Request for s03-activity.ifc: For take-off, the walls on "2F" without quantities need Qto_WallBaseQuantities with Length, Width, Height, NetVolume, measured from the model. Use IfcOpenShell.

First a look at what the model holds.

```python
import ifcopenshell
import ifcopenshell.util.element
import ifcopenshell.util.unit

model = ifcopenshell.open("s03-activity.ifc")
print(model.schema)
for unit_type in ("LENGTHUNIT", "AREAUNIT", "VOLUMEUNIT"):
    print(unit_type, ifcopenshell.util.unit.calculate_unit_scale(model, unit_type))
storey = next(s for s in model.by_type("IfcBuildingStorey") if s.Name == "2F")
walls = [e for e in ifcopenshell.util.element.get_decomposition(storey) if e.is_a("IfcWall")]
for e in sorted(walls, key=lambda e: e.id()):
    print(e.id(), e.is_a(), e.Name, list(ifcopenshell.util.element.get_psets(e, qtos_only=True)), sep=" | ")
```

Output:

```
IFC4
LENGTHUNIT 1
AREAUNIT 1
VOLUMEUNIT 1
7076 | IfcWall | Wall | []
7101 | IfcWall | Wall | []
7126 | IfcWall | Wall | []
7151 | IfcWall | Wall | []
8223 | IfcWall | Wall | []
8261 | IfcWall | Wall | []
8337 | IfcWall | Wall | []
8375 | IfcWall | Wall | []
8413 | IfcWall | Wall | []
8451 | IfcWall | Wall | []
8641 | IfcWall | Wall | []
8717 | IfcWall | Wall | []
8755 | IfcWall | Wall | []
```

```python
import ifcopenshell
import ifcopenshell.api.pset
import ifcopenshell.geom
import ifcopenshell.util.element
import ifcopenshell.util.shape
import ifcopenshell.util.unit

model = ifcopenshell.open("s03-activity.ifc")
unit_scale = ifcopenshell.util.unit.calculate_unit_scale(model)
volume_scale = ifcopenshell.util.unit.calculate_unit_scale(model, "VOLUMEUNIT")
settings = ifcopenshell.geom.settings()

storey = next(s for s in model.by_type("IfcBuildingStorey") if s.Name == "2F")
walls = [e for e in ifcopenshell.util.element.get_decomposition(storey) if e.is_a("IfcWall")]

for e in sorted(walls, key=lambda e: e.id()):
    if ifcopenshell.util.element.get_psets(e, qtos_only=True, should_inherit=False):
        continue
    # Geometry comes back in metres, in the element's own axes.
    shape = ifcopenshell.geom.create_shape(settings, e)
    values = {
        "Length": ifcopenshell.util.shape.get_x(shape.geometry) / unit_scale,
        "Width": ifcopenshell.util.shape.get_y(shape.geometry) / unit_scale,
        "Height": ifcopenshell.util.shape.get_z(shape.geometry) / unit_scale,
        "NetVolume": ifcopenshell.util.shape.get_volume(shape.geometry) / volume_scale,
    }
    qto = ifcopenshell.api.pset.add_qto(model, product=e, name="Qto_WallBaseQuantities")
    ifcopenshell.api.pset.edit_qto(model, qto=qto, properties=values)
    print(e.id(), {k: round(v, 3) for k, v in values.items()})

model.write("s03-activity_edited.ifc")
```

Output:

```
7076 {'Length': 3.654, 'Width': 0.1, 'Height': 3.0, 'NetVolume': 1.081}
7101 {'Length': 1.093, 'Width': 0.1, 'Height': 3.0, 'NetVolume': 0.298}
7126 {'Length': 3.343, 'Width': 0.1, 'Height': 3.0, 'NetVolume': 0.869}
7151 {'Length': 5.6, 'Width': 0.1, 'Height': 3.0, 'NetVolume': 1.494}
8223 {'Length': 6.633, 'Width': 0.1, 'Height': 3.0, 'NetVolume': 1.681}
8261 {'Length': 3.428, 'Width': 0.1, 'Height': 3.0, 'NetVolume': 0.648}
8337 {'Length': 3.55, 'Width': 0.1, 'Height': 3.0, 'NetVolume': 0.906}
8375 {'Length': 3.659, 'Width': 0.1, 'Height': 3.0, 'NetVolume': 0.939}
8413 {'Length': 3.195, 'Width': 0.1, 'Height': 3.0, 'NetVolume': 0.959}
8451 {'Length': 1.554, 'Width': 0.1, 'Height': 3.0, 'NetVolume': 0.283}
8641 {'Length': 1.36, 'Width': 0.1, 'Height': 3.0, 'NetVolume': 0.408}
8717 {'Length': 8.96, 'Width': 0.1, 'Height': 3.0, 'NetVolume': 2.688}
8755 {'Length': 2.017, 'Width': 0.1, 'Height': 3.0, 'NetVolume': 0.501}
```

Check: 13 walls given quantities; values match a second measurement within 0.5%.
